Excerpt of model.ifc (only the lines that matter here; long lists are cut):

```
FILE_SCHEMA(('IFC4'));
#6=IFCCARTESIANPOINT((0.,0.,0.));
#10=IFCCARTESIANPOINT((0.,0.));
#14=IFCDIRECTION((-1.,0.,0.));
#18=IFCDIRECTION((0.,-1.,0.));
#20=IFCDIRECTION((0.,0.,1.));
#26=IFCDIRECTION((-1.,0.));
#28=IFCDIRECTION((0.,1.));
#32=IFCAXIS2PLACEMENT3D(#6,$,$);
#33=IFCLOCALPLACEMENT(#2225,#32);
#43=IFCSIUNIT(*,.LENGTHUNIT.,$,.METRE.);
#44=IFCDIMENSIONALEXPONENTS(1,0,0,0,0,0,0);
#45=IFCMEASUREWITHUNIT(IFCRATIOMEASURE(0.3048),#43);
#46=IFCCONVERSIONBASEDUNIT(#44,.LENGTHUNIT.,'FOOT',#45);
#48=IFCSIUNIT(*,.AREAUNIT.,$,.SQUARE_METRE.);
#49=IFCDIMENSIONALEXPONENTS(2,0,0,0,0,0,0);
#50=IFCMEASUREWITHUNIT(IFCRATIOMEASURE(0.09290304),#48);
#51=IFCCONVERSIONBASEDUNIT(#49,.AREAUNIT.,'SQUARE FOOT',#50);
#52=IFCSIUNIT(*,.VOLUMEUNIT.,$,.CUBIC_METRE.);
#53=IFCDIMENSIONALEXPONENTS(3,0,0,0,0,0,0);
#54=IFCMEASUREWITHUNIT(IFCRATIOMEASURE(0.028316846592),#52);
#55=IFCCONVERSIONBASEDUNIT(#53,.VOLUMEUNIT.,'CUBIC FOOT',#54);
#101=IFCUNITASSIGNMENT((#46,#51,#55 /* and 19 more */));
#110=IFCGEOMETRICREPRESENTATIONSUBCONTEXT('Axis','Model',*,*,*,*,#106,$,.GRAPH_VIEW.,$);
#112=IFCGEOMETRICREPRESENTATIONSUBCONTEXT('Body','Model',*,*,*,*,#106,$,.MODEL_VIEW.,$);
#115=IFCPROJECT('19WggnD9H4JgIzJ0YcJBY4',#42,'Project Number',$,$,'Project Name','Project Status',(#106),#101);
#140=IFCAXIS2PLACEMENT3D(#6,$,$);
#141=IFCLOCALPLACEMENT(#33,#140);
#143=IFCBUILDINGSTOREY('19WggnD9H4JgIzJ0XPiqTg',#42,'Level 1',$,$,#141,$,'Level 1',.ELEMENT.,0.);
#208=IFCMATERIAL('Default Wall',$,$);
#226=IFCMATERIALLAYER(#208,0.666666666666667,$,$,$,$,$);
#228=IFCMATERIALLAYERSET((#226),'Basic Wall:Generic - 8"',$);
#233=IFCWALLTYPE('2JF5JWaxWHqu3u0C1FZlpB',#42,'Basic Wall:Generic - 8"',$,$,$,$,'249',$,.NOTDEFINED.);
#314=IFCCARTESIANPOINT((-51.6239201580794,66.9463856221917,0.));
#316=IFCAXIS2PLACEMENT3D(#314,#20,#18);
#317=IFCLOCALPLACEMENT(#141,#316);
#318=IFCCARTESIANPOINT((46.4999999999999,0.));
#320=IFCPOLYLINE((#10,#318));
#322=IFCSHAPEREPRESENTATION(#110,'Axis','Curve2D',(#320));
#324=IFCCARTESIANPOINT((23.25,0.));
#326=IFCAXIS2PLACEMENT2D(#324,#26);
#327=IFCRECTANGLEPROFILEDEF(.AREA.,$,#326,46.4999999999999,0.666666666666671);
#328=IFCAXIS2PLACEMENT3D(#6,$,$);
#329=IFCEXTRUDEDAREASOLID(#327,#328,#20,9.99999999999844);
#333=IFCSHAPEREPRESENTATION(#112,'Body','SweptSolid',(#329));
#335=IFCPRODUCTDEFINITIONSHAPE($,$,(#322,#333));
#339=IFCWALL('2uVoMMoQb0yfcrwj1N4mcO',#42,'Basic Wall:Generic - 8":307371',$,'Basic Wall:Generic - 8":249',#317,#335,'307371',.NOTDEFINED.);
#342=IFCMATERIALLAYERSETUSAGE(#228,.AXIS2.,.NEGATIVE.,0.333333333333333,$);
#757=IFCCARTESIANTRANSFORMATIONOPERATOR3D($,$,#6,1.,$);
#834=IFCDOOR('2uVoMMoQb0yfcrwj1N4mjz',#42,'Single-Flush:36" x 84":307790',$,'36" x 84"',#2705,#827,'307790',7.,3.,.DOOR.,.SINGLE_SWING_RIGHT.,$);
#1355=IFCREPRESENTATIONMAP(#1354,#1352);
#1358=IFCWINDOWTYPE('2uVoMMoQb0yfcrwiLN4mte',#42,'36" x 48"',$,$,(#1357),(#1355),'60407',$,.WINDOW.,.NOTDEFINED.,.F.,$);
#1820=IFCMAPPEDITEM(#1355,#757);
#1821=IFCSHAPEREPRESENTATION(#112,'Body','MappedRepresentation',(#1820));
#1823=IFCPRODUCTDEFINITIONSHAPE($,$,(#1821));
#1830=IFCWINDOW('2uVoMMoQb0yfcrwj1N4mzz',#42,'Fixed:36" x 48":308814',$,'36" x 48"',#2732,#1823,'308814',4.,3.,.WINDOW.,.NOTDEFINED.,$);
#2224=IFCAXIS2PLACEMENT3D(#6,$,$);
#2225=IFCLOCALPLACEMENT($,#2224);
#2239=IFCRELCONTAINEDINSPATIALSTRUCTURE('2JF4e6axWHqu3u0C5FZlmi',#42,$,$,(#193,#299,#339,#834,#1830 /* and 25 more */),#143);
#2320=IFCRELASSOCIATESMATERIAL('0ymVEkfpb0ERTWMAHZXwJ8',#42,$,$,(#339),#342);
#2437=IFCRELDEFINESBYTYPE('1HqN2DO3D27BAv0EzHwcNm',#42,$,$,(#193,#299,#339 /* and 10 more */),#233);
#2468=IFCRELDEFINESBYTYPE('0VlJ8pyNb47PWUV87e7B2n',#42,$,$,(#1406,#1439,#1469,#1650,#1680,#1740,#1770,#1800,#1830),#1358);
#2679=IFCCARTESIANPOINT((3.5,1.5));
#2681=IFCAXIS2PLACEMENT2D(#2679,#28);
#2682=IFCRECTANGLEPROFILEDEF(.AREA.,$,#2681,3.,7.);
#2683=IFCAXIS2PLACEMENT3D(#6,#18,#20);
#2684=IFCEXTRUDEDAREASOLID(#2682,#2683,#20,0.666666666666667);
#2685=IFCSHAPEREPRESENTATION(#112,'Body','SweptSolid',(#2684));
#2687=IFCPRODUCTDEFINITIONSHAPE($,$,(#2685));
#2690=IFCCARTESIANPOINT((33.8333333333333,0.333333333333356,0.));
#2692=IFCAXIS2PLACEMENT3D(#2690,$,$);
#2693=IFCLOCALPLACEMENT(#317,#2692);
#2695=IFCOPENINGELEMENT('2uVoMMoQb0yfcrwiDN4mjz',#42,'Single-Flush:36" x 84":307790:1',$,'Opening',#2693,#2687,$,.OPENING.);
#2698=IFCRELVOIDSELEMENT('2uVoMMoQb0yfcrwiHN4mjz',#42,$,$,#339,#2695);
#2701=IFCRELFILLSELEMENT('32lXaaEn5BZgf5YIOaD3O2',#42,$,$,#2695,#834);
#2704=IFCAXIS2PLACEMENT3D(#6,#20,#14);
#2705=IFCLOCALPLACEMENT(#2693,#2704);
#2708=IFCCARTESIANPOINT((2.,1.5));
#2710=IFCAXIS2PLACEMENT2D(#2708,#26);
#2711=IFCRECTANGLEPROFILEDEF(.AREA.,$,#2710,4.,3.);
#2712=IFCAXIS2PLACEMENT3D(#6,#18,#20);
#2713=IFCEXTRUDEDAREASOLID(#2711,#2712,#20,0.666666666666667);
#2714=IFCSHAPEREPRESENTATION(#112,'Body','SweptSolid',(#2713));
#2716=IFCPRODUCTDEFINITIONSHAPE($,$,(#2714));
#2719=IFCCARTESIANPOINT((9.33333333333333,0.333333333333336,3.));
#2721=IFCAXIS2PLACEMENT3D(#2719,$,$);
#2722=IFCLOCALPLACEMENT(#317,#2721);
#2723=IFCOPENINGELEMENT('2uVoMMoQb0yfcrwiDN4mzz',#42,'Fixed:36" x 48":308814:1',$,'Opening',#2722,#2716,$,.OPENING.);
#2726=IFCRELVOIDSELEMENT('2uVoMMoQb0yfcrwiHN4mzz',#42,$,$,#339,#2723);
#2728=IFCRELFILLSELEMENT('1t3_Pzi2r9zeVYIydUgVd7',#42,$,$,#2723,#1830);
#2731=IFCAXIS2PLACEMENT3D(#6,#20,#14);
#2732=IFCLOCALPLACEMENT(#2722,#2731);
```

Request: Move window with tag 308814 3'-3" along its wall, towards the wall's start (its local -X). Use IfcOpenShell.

```python
import ifcopenshell
import ifcopenshell.api.geometry
import ifcopenshell.util.placement
import ifcopenshell.util.unit

model = ifcopenshell.open("model.ifc")
unit_scale = ifcopenshell.util.unit.calculate_unit_scale(model)

window = model.by_guid("2uVoMMoQb0yfcrwj1N4mzz")
opening = window.FillsVoids[0].RelatingOpeningElement
wall = opening.VoidsElements[0].RelatingBuildingElement

wall_matrix = ifcopenshell.util.placement.get_local_placement(wall.ObjectPlacement)
shift = wall_matrix[:3, 0] * -39 * 0.0254 / unit_scale
before = ifcopenshell.util.placement.get_local_placement(window.ObjectPlacement)[:3, 3].copy()

# The window is placed relative to its opening, so it follows when the opening moves.
matrix = ifcopenshell.util.placement.get_local_placement(opening.ObjectPlacement)
matrix[:3, 3] += shift
ifcopenshell.api.geometry.edit_object_placement(
    model, product=opening, matrix=matrix, is_si=False, should_transform_children=True
)

after = ifcopenshell.util.placement.get_local_placement(window.ObjectPlacement)[:3, 3]
print("window moved by", (after - before).round(3) + 0.0)

model.write("model_edited.ifc")
```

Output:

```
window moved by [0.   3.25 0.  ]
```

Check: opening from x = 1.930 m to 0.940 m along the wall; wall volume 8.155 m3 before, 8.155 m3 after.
